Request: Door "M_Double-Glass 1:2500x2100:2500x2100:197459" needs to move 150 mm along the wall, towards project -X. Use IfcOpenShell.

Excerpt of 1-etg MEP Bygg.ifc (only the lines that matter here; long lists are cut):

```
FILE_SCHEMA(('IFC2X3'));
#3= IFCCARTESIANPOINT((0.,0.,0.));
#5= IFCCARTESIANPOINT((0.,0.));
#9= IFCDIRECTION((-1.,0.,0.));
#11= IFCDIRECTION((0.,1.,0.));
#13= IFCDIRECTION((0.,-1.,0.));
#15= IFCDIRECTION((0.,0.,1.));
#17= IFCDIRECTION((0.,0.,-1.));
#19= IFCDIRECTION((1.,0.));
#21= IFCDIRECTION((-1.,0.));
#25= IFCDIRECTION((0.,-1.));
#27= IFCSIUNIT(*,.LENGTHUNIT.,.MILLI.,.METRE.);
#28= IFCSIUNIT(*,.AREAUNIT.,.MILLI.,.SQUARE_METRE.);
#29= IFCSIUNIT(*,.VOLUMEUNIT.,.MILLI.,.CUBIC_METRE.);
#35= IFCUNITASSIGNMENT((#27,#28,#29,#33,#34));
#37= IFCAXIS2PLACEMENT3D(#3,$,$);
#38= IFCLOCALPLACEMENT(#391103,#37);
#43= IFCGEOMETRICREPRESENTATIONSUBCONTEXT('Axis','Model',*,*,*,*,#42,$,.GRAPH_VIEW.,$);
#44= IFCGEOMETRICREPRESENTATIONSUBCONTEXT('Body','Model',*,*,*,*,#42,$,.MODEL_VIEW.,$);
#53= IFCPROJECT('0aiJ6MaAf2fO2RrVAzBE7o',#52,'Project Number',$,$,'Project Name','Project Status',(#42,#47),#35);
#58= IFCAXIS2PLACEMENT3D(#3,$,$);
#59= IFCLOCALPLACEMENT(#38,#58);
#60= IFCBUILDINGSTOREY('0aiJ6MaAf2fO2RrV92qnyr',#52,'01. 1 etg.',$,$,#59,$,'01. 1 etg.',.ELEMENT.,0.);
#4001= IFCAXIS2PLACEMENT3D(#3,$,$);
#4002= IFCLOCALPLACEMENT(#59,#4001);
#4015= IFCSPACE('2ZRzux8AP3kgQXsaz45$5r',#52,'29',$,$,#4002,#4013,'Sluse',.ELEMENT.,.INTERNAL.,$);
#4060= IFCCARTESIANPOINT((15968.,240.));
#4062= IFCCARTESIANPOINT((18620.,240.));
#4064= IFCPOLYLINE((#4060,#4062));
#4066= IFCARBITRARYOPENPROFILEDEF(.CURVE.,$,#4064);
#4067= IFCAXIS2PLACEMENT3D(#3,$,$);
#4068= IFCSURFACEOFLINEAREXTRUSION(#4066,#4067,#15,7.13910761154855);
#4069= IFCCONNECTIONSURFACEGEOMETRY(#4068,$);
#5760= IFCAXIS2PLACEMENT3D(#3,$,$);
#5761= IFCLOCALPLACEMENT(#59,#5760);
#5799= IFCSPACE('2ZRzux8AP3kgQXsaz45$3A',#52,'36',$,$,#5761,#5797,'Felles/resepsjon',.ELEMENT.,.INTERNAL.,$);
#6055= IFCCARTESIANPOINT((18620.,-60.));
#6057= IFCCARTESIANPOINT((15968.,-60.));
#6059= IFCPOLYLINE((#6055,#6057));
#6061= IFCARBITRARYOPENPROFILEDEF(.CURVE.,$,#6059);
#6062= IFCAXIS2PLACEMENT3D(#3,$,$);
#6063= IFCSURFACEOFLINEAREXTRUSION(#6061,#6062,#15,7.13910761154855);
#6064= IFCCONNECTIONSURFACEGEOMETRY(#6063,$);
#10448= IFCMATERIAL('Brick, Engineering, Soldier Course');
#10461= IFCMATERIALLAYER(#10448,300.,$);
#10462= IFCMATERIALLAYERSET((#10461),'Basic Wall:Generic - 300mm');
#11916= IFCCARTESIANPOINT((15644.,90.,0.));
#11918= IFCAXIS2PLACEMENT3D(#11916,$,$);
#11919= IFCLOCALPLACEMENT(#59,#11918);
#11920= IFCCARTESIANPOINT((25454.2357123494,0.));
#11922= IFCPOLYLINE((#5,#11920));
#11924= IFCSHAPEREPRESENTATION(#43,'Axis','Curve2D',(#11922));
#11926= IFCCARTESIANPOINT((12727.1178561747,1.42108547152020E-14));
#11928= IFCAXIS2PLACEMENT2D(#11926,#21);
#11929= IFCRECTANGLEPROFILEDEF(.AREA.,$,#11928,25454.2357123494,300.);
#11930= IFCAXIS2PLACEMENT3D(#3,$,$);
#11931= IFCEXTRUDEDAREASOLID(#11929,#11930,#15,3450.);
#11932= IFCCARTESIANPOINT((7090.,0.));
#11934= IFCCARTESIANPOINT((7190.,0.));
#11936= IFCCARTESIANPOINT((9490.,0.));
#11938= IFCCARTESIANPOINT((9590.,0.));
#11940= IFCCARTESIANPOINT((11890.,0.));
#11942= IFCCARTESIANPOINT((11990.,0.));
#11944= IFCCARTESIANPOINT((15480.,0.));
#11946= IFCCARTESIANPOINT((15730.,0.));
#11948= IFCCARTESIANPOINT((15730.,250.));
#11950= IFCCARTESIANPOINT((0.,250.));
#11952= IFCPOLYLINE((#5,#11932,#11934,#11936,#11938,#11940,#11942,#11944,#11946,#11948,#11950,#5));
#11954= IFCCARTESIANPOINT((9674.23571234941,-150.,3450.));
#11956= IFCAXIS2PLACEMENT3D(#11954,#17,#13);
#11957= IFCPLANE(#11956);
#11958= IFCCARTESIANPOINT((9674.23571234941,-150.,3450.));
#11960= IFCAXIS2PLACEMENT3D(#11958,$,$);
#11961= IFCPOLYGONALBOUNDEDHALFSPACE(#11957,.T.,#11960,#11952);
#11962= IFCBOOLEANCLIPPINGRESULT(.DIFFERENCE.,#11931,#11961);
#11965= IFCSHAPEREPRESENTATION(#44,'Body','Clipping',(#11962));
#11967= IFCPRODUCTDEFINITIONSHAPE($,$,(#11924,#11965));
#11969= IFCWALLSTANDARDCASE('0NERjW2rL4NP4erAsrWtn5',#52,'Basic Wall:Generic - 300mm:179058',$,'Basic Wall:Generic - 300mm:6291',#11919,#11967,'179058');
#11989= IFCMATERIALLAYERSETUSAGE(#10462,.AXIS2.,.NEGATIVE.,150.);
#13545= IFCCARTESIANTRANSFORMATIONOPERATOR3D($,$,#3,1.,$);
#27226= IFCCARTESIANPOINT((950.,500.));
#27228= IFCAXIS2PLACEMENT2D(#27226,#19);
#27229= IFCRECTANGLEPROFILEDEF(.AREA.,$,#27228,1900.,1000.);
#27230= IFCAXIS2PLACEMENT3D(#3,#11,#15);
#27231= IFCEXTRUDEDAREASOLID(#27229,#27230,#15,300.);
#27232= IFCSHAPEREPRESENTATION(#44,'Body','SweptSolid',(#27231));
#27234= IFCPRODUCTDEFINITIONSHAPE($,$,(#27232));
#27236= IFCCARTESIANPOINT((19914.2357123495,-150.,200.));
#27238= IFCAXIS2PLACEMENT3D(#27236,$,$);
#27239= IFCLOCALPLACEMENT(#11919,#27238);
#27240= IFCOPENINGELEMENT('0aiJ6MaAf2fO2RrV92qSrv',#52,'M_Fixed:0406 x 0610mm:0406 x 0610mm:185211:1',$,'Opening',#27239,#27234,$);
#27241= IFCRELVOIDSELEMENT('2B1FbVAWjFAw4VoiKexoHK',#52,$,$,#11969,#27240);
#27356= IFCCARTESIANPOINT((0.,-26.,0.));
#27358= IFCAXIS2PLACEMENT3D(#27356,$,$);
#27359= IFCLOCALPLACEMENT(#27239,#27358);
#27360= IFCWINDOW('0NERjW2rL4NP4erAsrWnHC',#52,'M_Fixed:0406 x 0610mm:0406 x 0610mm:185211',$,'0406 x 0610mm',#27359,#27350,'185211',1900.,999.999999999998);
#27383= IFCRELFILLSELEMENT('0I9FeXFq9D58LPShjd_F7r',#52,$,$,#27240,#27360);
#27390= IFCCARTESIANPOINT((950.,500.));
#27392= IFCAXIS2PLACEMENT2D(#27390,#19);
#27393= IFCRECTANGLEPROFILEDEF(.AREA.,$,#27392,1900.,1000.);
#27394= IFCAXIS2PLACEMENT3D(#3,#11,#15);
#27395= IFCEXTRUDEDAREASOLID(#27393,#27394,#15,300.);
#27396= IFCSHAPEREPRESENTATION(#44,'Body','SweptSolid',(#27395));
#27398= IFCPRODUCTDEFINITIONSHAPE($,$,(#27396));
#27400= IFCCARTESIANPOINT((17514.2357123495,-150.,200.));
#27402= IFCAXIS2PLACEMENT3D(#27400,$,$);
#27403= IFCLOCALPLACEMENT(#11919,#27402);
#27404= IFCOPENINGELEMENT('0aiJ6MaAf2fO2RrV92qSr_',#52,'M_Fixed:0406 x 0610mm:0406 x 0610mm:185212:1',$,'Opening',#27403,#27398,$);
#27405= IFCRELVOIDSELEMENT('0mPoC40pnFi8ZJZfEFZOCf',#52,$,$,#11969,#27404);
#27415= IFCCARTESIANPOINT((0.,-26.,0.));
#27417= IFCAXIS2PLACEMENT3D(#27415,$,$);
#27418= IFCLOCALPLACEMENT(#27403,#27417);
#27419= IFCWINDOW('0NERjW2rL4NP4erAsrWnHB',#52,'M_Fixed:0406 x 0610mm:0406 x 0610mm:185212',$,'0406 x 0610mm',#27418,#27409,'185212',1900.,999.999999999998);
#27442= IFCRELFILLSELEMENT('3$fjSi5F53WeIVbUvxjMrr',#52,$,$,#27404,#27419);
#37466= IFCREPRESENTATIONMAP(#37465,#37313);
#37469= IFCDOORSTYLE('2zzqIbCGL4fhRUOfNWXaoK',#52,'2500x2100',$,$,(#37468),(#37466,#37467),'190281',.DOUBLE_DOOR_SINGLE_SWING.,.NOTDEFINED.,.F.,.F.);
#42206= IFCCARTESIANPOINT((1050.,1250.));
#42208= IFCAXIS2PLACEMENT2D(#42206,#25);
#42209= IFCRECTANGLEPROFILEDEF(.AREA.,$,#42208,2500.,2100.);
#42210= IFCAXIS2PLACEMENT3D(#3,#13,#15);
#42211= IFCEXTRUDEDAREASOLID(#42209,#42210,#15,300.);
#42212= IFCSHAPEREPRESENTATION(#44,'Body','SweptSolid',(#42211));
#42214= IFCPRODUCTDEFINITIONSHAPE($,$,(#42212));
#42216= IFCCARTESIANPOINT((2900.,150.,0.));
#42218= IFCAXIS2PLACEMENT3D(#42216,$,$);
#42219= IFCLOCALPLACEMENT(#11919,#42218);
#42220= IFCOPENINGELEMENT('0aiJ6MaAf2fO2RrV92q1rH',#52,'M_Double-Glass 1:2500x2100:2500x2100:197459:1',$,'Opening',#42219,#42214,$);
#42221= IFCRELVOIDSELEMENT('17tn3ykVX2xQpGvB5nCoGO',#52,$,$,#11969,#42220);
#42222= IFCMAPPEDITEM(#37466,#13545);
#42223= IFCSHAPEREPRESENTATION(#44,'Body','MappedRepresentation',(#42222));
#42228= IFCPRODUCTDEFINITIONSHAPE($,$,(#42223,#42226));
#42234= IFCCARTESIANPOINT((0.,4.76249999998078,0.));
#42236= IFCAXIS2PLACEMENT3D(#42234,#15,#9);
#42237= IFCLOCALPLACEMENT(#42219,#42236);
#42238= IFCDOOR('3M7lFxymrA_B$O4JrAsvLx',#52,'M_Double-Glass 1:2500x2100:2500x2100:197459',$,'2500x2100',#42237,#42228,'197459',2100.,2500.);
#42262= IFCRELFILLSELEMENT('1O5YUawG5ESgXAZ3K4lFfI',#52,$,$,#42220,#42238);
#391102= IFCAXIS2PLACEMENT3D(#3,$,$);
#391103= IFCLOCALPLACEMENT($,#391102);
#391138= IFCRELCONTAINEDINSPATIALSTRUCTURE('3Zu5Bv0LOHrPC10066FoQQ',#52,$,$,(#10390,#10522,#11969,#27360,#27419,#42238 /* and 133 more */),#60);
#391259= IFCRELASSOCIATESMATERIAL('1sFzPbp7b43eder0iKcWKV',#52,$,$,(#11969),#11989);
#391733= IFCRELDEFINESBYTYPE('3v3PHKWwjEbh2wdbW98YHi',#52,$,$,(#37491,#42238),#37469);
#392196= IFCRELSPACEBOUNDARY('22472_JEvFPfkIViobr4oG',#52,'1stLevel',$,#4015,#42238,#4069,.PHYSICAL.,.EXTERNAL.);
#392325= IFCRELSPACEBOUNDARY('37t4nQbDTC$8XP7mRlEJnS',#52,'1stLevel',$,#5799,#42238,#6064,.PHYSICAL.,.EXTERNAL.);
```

```python
import numpy as np
import ifcopenshell
import ifcopenshell.api.geometry
import ifcopenshell.util.placement

model = ifcopenshell.open("1-etg MEP Bygg.ifc")

door = model.by_guid("3M7lFxymrA_B$O4JrAsvLx")
opening = door.FillsVoids[0].RelatingOpeningElement
wall = opening.VoidsElements[0].RelatingBuildingElement

wall_matrix = ifcopenshell.util.placement.get_local_placement(wall.ObjectPlacement)
shift = wall_matrix[:3, 0] * -150.0
before = ifcopenshell.util.placement.get_local_placement(door.ObjectPlacement)[:3, 3].copy()

# The door is placed relative to its opening, so it follows when the opening moves.
matrix = ifcopenshell.util.placement.get_local_placement(opening.ObjectPlacement)
matrix[:3, 3] += shift
ifcopenshell.api.geometry.edit_object_placement(
    model, product=opening, matrix=matrix, is_si=False, should_transform_children=True
)

# Space boundary surfaces are stored in each space's coordinates; move them too.
for rel in door.ProvidesBoundaries:
    if not rel.ConnectionGeometry:
        continue
    surface = rel.ConnectionGeometry.SurfaceOnRelatingElement
    space_matrix = ifcopenshell.util.placement.get_local_placement(rel.RelatingSpace.ObjectPlacement)
    point = np.array(surface.Position.Location.Coordinates) + space_matrix[:3, :3].T @ shift
    surface.Position = model.createIfcAxis2Placement3D(
        model.createIfcCartesianPoint(point.tolist()), surface.Position.Axis, surface.Position.RefDirection
    )

after = ifcopenshell.util.placement.get_local_placement(door.ObjectPlacement)[:3, 3]
print("door moved by", (after - before).round(3) + 0.0)

model.write("1-etg MEP Bygg_v2.ifc")
```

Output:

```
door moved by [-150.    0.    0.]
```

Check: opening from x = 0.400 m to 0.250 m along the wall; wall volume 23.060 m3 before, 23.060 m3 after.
